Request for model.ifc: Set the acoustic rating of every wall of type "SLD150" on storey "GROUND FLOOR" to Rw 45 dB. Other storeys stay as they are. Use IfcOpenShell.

First a look at what the model holds.

```python
import ifcopenshell
import ifcopenshell.util.element

model = ifcopenshell.open("model.ifc")
print(model.schema)
storey = next(s for s in model.by_type("IfcBuildingStorey") if s.Name == "GROUND FLOOR")
walls = [e for e in ifcopenshell.util.element.get_decomposition(storey) if e.is_a("IfcWall")]
seen = {}
for e in walls:
    element_type = ifcopenshell.util.element.get_type(e)
    key = (element_type.Name if element_type != e and element_type else None, ifcopenshell.util.element.get_pset(e, "Pset_WallCommon", "AcousticRating"))
    seen[key] = seen.get(key, 0) + 1
for (name, value), count in sorted(seen.items(), key=str):
    print(count, "x", name, "|", value)
```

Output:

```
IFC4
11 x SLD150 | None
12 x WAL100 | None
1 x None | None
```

```python
import ifcopenshell
import ifcopenshell.api.pset
import ifcopenshell.util.element

model = ifcopenshell.open("model.ifc")

storey = next(s for s in model.by_type("IfcBuildingStorey") if s.Name == "GROUND FLOOR")
walls = [e for e in ifcopenshell.util.element.get_decomposition(storey) if e.is_a("IfcWall")]

count = 0
for e in walls:
    element_type = ifcopenshell.util.element.get_type(e)
    if element_type in (None, e) or element_type.Name != "SLD150":
        continue
    # add_pset returns the element's existing set when there is one.
    pset = ifcopenshell.api.pset.add_pset(model, product=e, name="Pset_WallCommon")
    ifcopenshell.api.pset.edit_pset(model, pset=pset, properties={"AcousticRating": "Rw 45 dB"})
    count += 1

print(count, "walls updated")

model.write("model-out.ifc")
```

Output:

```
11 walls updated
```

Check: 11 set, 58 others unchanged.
